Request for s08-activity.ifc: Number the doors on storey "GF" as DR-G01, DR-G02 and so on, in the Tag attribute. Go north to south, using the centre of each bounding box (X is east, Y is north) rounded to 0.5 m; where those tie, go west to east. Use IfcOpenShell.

First a look at what the model holds.

```python
import ifcopenshell
import ifcopenshell.util.element
import ifcopenshell.util.placement

model = ifcopenshell.open("s08-activity.ifc")
print(model.schema)
storey = next(s for s in model.by_type("IfcBuildingStorey") if s.Name == "GF")
doors = [e for e in ifcopenshell.util.element.get_decomposition(storey) if e.is_a("IfcDoor")]
for e in sorted(doors, key=lambda e: e.id()):
    origin = ifcopenshell.util.placement.get_local_placement(e.ObjectPlacement)[:3, 3]
    print(e.id(), e.Tag, e.Name, origin.round(2) + 0.0, sep=" | ")
```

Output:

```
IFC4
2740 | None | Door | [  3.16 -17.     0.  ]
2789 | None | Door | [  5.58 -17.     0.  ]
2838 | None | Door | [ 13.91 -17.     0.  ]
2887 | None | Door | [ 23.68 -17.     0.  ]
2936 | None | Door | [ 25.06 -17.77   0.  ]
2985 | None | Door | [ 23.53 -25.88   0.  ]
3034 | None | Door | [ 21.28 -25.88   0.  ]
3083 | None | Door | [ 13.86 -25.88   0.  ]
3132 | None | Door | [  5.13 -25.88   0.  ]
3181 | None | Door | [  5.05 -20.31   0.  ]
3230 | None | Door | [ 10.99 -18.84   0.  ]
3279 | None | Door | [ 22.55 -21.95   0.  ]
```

```python
import ifcopenshell
import ifcopenshell.geom
import ifcopenshell.util.element
import ifcopenshell.util.shape

model = ifcopenshell.open("s08-activity.ifc")
settings = ifcopenshell.geom.settings()
settings.set("use-world-coords", True)


def centre(element):
    shape = ifcopenshell.geom.create_shape(settings, element)
    return ifcopenshell.util.shape.get_bbox_centroid(shape.geometry)


storey = next(s for s in model.by_type("IfcBuildingStorey") if s.Name == "GF")
doors = [e for e in ifcopenshell.util.element.get_decomposition(storey) if e.is_a("IfcDoor")]

# Insertion points can sit at a corner or the storey origin, so sort by the geometry (in metres).
centres = {e: centre(e) for e in doors}
doors.sort(key=lambda e: (-round(centres[e][1] / 0.5), centres[e][0]))

for i, e in enumerate(doors, start=1):
    number = f"DR-G{i:02d}"
    e.Tag = number
    print(e.id(), number)

model.write("s08-activity_edited.ifc")
```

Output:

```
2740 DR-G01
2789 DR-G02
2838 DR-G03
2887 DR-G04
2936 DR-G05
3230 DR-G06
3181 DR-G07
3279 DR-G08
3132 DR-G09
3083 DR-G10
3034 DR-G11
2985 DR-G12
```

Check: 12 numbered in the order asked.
